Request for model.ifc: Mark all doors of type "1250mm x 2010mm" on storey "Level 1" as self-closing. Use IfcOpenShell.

First a look at what the model holds.

```python
import ifcopenshell
import ifcopenshell.util.element

model = ifcopenshell.open("model.ifc")
print(model.schema)
storey = next(s for s in model.by_type("IfcBuildingStorey") if s.Name == "Level 1")
doors = [e for e in ifcopenshell.util.element.get_decomposition(storey) if e.is_a("IfcDoor")]
seen = {}
for e in doors:
    element_type = ifcopenshell.util.element.get_type(e)
    key = (element_type.Name if element_type != e and element_type else None, ifcopenshell.util.element.get_pset(e, "Pset_DoorCommon", "SelfClosing"))
    seen[key] = seen.get(key, 0) + 1
for (name, value), count in sorted(seen.items(), key=str):
    print(count, "x", name, "|", value)
```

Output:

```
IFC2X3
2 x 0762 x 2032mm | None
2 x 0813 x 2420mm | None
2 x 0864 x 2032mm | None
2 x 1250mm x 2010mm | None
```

```python
import ifcopenshell
import ifcopenshell.api.pset
import ifcopenshell.util.element

model = ifcopenshell.open("model.ifc")

storey = next(s for s in model.by_type("IfcBuildingStorey") if s.Name == "Level 1")
doors = [e for e in ifcopenshell.util.element.get_decomposition(storey) if e.is_a("IfcDoor")]

count = 0
for e in doors:
    element_type = ifcopenshell.util.element.get_type(e)
    if element_type in (None, e) or element_type.Name != "1250mm x 2010mm":
        continue
    # add_pset returns the element's existing set when there is one.
    pset = ifcopenshell.api.pset.add_pset(model, product=e, name="Pset_DoorCommon")
    ifcopenshell.api.pset.edit_pset(model, pset=pset, properties={"SelfClosing": True})
    count += 1

print(count, "doors updated")

model.write("model-out.ifc")
```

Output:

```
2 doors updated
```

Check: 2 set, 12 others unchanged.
